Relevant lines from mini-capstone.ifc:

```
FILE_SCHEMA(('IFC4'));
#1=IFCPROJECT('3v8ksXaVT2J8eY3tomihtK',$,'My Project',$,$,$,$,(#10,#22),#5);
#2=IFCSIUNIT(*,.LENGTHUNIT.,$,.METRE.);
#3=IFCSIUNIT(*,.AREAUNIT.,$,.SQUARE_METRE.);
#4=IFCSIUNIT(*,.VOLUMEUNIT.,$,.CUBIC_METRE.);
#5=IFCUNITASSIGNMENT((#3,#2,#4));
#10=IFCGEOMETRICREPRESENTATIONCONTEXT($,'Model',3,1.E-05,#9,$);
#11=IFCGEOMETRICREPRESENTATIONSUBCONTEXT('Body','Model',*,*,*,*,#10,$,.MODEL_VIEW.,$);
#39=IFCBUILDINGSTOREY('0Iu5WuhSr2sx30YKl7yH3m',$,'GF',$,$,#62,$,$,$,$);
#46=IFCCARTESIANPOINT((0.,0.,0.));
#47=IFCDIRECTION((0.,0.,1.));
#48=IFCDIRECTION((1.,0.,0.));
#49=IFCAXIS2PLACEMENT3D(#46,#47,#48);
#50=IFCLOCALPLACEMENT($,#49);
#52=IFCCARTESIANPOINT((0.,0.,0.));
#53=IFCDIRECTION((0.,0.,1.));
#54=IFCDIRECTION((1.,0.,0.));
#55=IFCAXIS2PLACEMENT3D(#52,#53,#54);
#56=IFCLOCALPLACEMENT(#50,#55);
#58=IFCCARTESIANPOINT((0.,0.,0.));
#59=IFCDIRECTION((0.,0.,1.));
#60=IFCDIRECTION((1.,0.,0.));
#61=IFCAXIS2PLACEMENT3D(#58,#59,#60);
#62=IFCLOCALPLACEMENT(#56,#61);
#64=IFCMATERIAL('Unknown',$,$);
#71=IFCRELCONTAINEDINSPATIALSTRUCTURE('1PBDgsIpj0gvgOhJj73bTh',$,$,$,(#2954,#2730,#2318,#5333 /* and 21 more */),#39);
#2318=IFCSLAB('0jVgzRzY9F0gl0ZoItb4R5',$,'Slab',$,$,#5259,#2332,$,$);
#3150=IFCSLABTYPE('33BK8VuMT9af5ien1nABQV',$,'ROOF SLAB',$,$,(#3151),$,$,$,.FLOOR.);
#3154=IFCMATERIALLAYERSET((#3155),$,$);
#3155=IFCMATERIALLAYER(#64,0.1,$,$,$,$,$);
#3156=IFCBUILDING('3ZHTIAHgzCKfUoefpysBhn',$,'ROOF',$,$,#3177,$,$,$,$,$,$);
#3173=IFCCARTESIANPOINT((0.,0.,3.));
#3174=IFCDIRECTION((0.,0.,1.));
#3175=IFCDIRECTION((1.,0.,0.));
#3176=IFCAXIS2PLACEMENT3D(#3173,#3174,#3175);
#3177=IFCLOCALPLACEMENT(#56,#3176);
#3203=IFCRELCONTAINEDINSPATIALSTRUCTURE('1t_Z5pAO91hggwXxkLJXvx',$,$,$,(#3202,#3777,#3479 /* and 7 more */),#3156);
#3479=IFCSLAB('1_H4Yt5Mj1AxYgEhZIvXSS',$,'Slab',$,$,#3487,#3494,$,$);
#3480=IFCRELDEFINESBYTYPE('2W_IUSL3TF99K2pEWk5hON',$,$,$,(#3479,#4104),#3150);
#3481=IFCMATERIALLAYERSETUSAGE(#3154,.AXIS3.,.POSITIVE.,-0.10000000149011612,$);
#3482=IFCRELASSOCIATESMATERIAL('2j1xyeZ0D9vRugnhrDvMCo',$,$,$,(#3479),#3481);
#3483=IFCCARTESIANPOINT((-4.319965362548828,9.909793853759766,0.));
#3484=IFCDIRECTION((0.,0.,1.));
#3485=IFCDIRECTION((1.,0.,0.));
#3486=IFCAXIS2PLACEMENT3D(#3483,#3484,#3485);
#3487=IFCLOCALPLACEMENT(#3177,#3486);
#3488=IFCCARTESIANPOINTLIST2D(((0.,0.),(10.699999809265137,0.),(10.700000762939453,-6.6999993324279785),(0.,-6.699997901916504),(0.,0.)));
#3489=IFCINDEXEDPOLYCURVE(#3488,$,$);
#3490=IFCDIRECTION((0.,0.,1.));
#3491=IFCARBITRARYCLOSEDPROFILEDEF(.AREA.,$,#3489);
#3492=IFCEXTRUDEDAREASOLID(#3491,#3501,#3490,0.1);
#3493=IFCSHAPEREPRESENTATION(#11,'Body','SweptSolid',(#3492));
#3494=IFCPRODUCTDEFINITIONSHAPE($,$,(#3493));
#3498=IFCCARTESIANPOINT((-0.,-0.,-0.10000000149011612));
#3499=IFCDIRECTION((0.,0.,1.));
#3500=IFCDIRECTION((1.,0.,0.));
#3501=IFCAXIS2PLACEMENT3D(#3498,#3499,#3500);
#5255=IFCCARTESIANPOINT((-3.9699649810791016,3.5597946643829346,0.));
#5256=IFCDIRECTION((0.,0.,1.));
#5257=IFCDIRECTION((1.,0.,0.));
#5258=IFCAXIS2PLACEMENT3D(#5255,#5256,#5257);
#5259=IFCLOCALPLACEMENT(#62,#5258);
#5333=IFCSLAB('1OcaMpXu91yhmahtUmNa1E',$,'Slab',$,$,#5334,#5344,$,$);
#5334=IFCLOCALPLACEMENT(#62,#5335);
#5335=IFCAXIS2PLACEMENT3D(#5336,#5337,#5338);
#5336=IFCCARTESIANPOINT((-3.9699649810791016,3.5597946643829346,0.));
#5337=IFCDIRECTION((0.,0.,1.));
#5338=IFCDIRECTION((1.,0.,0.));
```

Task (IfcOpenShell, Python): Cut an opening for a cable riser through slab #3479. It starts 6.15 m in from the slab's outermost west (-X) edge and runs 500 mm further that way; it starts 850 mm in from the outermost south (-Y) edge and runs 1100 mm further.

```python
import numpy as np
import ifcopenshell
import ifcopenshell.api.feature
import ifcopenshell.api.geometry
import ifcopenshell.api.root
import ifcopenshell.geom
import ifcopenshell.util.placement
import ifcopenshell.util.representation
import ifcopenshell.util.shape
import ifcopenshell.util.unit

model = ifcopenshell.open("mini-capstone.ifc")
unit_scale = ifcopenshell.util.unit.calculate_unit_scale(model)
settings = ifcopenshell.geom.settings()


def volume(element):
    """Net volume in cubic metres, openings subtracted."""
    shape = ifcopenshell.geom.create_shape(settings, element)
    return ifcopenshell.util.shape.get_volume(shape.geometry)


slab = model.by_guid("1_H4Yt5Mj1AxYgEhZIvXSS")
before = volume(slab)

# Extent in the slab's own axes, in metres. The edges named are its -X and -Y sides.
slab_shape = ifcopenshell.geom.create_shape(settings, slab)
vertices = ifcopenshell.util.shape.get_vertices(slab_shape.geometry)
x_min, y_min, bottom = vertices.min(axis=0)
top = vertices[:, 2].max()

opening = ifcopenshell.api.root.create_entity(model, ifc_class="IfcOpeningElement", name="Cable riser opening", predefined_type="OPENING")
context = ifcopenshell.util.representation.get_context(model, "Model", "Body", "MODEL_VIEW")
width, depth = 0.5, 1.1
outline = [(0.0, 0.0), (width, 0.0), (width, depth), (0.0, depth), (0.0, 0.0)]
# Overshoot both faces by 50 mm so the cut is clean.
shape = ifcopenshell.api.geometry.add_slab_representation(
    model, context=context, depth=top - bottom + 0.1, polyline=outline
)
ifcopenshell.api.geometry.assign_representation(model, product=opening, representation=shape)

matrix = ifcopenshell.util.placement.get_local_placement(slab.ObjectPlacement)
matrix[:, 3] = matrix @ np.append(np.array([x_min + 6.15, y_min + 0.85, bottom - 0.05]) / unit_scale, 1.0)
ifcopenshell.api.geometry.edit_object_placement(model, product=opening, matrix=matrix, is_si=False)
ifcopenshell.api.feature.add_feature(model, feature=opening, element=slab)

after = volume(slab)

print(f"slab volume {before:.3f} -> {after:.3f} m3")

model.write("mini-capstone_v2.ifc")
```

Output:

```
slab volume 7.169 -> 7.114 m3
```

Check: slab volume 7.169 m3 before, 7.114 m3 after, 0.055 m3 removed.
